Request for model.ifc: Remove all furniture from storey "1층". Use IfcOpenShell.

First a look at what the model holds.

```python
import ifcopenshell
import ifcopenshell.util.element

model = ifcopenshell.open("model.ifc")
print(model.schema)
storey = next(s for s in model.by_type("IfcBuildingStorey") if s.Name == "1층")
furniture = [e for e in ifcopenshell.util.element.get_decomposition(storey) if e.is_a("IfcFurnishingElement")]
seen = {}
for e in furniture:
    element_type = ifcopenshell.util.element.get_type(e)
    name = element_type.Name if element_type not in (None, e) else None
    seen[name] = seen.get(name, 0) + 1
for name, count in sorted(seen.items(), key=str):
    print(count, "x", name)
```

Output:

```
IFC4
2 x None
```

```python
import ifcopenshell
import ifcopenshell.api.root
import ifcopenshell.util.element

model = ifcopenshell.open("model.ifc")

storey = next(s for s in model.by_type("IfcBuildingStorey") if s.Name == "1층")
furniture = [e for e in ifcopenshell.util.element.get_decomposition(storey) if e.is_a("IfcFurnishingElement")]

for e in furniture:
    ifcopenshell.api.root.remove_product(model, product=e)
print(len(furniture), "removed")

model.write("model_edited.ifc")
```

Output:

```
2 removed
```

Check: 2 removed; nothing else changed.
